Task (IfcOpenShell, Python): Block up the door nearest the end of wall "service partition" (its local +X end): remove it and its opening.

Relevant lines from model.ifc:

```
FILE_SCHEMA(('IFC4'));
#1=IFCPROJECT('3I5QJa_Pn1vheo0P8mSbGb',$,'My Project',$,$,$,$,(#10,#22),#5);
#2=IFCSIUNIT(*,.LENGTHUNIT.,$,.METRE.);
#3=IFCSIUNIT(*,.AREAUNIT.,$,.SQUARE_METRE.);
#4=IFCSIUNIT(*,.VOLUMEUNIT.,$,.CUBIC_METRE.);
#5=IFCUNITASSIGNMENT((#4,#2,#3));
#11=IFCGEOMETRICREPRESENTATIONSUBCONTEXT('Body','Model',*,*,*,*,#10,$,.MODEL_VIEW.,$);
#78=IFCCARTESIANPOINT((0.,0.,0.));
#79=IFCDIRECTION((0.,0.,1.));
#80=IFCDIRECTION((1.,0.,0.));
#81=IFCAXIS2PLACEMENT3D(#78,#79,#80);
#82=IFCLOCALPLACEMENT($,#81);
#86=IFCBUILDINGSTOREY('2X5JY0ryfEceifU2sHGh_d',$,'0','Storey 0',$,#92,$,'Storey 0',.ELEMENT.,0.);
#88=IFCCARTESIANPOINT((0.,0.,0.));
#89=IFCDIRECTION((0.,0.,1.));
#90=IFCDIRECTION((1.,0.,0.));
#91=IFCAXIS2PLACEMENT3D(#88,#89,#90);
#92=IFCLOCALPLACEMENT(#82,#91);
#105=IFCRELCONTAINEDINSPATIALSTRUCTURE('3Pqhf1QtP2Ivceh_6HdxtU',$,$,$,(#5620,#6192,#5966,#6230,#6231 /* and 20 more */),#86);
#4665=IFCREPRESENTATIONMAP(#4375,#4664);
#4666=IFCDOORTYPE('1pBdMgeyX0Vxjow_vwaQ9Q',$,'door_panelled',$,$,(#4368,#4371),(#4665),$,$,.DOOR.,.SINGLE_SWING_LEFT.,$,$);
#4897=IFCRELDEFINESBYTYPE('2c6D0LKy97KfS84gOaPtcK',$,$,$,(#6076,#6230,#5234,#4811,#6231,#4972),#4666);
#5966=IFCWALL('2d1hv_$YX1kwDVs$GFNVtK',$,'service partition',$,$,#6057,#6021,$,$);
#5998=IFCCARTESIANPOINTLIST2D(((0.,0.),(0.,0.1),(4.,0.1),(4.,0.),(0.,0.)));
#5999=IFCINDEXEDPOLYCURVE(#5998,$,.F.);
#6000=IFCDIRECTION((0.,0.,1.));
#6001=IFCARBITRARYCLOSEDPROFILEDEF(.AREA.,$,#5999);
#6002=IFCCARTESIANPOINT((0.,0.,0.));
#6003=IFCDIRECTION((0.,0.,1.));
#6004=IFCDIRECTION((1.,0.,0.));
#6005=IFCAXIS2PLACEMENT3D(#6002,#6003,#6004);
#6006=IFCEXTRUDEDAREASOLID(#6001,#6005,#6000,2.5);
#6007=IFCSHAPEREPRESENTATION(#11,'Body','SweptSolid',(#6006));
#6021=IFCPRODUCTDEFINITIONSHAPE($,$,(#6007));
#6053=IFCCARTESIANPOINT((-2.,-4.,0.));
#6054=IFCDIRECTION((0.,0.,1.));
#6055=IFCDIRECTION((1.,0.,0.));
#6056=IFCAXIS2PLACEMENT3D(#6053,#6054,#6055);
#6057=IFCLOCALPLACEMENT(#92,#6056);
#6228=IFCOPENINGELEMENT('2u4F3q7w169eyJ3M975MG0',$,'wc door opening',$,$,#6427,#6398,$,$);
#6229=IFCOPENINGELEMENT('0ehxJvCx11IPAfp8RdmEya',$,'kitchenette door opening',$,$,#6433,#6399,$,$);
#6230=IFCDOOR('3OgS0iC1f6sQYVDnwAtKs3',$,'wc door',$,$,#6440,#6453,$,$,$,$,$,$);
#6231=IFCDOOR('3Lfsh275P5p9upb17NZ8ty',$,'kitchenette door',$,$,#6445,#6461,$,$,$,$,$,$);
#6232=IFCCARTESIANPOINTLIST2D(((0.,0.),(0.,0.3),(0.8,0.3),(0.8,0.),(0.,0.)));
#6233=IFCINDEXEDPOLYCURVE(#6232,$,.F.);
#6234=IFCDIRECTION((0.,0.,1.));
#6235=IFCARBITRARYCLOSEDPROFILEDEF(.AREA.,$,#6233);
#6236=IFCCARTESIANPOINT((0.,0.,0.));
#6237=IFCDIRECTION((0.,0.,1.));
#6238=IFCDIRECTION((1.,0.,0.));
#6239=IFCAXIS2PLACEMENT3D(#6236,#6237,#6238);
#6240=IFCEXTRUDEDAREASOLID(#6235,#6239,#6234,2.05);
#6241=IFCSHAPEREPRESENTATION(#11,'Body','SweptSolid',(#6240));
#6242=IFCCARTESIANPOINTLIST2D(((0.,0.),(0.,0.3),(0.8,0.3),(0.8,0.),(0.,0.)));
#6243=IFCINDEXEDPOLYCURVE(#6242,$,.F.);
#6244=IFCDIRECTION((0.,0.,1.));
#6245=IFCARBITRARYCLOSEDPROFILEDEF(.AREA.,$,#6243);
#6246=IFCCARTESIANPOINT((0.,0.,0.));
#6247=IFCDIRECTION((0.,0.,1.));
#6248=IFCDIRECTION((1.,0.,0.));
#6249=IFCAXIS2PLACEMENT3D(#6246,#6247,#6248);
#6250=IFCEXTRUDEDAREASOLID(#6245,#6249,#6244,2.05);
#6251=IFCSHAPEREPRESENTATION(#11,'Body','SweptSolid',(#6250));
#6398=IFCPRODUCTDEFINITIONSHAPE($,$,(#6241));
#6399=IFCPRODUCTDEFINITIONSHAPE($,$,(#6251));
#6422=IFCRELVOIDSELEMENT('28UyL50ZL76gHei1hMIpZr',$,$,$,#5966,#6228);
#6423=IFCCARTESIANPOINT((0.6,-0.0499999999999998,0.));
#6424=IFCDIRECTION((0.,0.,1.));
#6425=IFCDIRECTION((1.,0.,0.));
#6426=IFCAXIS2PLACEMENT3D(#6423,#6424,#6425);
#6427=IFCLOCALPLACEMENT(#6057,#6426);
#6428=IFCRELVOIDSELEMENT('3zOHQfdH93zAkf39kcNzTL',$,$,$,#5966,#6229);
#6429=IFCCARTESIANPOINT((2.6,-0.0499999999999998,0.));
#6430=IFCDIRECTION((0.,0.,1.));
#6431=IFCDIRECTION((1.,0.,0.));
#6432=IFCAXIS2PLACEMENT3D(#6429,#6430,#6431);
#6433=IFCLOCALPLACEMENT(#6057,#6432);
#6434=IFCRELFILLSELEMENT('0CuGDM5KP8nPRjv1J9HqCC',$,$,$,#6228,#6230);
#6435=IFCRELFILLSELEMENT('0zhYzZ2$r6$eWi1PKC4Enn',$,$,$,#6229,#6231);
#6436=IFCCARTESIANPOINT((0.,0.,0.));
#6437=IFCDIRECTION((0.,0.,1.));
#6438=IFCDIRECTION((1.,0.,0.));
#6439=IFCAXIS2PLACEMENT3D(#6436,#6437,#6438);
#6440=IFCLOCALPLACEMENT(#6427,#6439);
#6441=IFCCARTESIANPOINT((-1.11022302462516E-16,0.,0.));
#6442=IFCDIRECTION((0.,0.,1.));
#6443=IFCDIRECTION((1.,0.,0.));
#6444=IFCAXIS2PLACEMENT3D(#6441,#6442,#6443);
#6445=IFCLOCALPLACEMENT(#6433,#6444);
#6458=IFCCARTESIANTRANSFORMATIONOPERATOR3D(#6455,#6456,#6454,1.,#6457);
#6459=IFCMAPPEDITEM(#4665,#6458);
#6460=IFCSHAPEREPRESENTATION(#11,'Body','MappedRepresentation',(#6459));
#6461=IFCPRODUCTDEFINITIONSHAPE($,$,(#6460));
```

```python
import ifcopenshell
import ifcopenshell.api.feature
import ifcopenshell.api.root
import ifcopenshell.geom
import ifcopenshell.util.shape

model = ifcopenshell.open("model.ifc")
settings = ifcopenshell.geom.settings()


def volume(element):
    """Net volume in cubic metres, openings subtracted."""
    shape = ifcopenshell.geom.create_shape(settings, element)
    return ifcopenshell.util.shape.get_volume(shape.geometry)


door = model.by_id(6231)
opening = door.FillsVoids[0].RelatingOpeningElement
wall = opening.VoidsElements[0].RelatingBuildingElement
before = volume(wall)

ifcopenshell.api.root.remove_product(model, product=door)
ifcopenshell.api.feature.remove_feature(model, feature=opening)

after = volume(wall)

print(f"wall volume {before:.3f} -> {after:.3f} m3")

model.write("model-out.ifc")
```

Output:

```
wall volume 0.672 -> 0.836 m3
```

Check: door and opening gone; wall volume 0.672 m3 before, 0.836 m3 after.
